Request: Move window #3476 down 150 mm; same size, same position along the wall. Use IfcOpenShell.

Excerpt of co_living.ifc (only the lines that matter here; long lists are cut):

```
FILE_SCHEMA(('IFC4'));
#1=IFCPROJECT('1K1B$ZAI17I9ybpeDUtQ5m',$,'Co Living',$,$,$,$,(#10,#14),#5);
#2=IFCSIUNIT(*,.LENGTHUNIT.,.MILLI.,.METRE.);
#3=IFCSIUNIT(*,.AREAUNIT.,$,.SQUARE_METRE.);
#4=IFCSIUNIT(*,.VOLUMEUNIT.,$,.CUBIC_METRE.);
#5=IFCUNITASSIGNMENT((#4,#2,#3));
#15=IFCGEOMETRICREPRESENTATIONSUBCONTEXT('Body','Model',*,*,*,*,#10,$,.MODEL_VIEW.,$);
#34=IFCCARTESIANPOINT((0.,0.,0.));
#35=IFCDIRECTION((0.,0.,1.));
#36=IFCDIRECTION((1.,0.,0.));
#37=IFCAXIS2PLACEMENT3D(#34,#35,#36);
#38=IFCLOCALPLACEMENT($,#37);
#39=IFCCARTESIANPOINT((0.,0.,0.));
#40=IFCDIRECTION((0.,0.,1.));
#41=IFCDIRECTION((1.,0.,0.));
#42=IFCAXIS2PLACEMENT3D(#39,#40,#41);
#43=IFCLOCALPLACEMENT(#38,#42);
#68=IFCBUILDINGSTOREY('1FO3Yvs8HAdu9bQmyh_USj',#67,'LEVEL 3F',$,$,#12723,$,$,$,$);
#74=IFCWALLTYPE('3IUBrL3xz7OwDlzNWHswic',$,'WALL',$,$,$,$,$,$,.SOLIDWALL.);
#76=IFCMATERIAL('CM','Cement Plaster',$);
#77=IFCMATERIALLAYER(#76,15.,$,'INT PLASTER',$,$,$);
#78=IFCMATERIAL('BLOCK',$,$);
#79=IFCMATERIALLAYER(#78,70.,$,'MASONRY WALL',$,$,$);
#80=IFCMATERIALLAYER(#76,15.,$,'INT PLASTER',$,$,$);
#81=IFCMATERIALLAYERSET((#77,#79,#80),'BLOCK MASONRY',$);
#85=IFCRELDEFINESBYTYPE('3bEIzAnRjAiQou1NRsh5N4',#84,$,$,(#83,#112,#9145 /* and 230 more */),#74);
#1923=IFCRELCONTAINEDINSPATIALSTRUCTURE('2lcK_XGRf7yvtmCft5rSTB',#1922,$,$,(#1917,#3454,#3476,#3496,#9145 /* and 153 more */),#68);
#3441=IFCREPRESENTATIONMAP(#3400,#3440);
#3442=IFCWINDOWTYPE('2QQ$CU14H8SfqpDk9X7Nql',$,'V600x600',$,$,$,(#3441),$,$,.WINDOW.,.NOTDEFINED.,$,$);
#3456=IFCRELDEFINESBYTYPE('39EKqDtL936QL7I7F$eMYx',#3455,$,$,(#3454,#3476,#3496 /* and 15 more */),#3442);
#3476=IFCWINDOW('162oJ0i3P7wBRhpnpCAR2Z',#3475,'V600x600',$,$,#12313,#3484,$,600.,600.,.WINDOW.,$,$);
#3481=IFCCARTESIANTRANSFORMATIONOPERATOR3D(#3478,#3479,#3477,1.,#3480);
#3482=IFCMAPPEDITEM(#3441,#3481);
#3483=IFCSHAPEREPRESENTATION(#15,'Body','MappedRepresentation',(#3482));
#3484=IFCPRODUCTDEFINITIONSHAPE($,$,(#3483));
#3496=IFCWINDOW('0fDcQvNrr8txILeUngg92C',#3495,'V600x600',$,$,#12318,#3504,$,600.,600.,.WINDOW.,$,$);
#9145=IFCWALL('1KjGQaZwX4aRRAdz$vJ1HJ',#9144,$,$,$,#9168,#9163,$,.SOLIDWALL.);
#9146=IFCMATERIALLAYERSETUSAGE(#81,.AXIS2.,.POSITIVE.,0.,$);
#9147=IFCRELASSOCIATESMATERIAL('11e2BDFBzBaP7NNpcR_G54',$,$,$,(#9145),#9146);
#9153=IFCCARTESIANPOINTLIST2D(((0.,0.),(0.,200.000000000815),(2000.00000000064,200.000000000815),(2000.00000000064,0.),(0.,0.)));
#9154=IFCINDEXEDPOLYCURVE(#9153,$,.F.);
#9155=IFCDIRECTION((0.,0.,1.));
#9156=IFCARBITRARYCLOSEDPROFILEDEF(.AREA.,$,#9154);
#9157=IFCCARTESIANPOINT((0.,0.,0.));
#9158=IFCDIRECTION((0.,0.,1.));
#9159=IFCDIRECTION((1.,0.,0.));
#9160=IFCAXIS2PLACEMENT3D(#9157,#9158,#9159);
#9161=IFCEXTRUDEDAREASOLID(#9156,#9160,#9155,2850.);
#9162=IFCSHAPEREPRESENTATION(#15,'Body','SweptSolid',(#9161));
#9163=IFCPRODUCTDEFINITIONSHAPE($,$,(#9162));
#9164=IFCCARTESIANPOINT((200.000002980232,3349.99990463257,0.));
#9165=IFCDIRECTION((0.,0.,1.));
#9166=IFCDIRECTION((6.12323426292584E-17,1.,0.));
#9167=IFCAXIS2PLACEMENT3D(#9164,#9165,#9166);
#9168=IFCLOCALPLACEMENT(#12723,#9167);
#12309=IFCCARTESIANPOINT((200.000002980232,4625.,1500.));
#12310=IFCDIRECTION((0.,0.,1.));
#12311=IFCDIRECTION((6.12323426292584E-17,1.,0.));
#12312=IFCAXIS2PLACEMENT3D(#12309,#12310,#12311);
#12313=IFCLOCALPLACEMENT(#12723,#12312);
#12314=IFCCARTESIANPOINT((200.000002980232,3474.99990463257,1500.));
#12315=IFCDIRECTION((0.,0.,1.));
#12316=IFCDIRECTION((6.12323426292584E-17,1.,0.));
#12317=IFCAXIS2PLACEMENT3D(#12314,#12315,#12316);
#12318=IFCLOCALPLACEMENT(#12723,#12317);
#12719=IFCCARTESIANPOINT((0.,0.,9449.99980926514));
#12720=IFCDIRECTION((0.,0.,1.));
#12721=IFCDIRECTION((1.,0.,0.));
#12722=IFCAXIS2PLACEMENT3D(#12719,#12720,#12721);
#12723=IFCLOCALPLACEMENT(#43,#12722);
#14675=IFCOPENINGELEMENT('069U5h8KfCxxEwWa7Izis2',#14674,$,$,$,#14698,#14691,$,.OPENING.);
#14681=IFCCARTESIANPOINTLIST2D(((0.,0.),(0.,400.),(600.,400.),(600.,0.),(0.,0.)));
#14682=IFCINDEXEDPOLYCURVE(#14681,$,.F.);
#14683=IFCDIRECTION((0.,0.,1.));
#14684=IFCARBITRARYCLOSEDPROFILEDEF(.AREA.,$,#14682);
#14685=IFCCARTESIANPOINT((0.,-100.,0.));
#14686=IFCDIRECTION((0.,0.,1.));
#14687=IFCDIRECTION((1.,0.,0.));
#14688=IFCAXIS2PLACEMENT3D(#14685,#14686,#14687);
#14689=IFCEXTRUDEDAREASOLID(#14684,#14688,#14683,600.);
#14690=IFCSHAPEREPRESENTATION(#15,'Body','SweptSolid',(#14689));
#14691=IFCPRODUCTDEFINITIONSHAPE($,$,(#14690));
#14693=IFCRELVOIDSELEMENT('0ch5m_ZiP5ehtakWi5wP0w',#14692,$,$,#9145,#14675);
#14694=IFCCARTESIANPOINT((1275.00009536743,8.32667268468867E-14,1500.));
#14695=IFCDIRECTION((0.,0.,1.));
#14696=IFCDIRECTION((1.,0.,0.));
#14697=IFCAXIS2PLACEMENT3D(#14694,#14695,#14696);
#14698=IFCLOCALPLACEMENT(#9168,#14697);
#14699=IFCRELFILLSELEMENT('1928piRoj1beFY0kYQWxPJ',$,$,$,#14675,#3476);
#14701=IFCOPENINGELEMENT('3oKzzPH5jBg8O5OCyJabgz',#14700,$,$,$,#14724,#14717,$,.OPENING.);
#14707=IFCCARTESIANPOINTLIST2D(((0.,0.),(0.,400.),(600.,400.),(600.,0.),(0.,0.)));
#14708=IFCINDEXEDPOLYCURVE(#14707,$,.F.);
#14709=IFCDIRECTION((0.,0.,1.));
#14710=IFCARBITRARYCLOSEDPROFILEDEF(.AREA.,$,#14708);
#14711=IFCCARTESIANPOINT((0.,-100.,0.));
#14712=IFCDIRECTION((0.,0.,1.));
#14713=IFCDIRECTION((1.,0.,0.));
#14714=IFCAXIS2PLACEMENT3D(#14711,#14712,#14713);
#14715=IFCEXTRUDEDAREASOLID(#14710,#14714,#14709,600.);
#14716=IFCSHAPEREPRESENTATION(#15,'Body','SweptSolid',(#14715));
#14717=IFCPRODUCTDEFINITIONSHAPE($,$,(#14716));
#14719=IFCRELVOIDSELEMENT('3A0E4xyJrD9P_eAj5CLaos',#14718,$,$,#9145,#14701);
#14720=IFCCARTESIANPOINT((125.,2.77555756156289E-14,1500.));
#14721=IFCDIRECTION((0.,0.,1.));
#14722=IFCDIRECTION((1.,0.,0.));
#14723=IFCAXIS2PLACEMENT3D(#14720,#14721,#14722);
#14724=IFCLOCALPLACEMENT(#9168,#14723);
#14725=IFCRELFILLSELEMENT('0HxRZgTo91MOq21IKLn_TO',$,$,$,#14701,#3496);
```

```python
import numpy as np
import ifcopenshell
import ifcopenshell.api.geometry
import ifcopenshell.util.placement
import ifcopenshell.util.unit

model = ifcopenshell.open("co_living.ifc")
unit_scale = ifcopenshell.util.unit.calculate_unit_scale(model)

window = model.by_guid("162oJ0i3P7wBRhpnpCAR2Z")
opening = window.FillsVoids[0].RelatingOpeningElement
dz = -0.15 / unit_scale

shift = np.array([0.0, 0.0, dz])
# The window is not placed relative to its opening, so move both.
for product in (opening, window):
    matrix = ifcopenshell.util.placement.get_local_placement(product.ObjectPlacement)
    matrix[:3, 3] += shift
    ifcopenshell.api.geometry.edit_object_placement(model, product=product, matrix=matrix, is_si=False)

print(f"moved by {dz * unit_scale:+.3f} m")

model.write("co_living-out.ifc")
```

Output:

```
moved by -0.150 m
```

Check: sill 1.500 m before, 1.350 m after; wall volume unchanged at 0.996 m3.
